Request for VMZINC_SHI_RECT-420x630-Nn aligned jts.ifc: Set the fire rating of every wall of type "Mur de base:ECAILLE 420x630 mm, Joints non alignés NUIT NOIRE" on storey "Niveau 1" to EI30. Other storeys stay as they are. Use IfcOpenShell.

First a look at what the model holds.

```python
import ifcopenshell
import ifcopenshell.util.element

model = ifcopenshell.open("VMZINC_SHI_RECT-420x630-Nn aligned jts.ifc")
print(model.schema)
storey = next(s for s in model.by_type("IfcBuildingStorey") if s.Name == "Niveau 1")
walls = [e for e in ifcopenshell.util.element.get_decomposition(storey) if e.is_a("IfcWall")]
seen = {}
for e in walls:
    element_type = ifcopenshell.util.element.get_type(e)
    key = (element_type.Name if element_type != e and element_type else None, ifcopenshell.util.element.get_pset(e, "Pset_WallCommon", "FireRating"))
    seen[key] = seen.get(key, 0) + 1
for (name, value), count in sorted(seen.items(), key=str):
    print(count, "x", name, "|", value)
```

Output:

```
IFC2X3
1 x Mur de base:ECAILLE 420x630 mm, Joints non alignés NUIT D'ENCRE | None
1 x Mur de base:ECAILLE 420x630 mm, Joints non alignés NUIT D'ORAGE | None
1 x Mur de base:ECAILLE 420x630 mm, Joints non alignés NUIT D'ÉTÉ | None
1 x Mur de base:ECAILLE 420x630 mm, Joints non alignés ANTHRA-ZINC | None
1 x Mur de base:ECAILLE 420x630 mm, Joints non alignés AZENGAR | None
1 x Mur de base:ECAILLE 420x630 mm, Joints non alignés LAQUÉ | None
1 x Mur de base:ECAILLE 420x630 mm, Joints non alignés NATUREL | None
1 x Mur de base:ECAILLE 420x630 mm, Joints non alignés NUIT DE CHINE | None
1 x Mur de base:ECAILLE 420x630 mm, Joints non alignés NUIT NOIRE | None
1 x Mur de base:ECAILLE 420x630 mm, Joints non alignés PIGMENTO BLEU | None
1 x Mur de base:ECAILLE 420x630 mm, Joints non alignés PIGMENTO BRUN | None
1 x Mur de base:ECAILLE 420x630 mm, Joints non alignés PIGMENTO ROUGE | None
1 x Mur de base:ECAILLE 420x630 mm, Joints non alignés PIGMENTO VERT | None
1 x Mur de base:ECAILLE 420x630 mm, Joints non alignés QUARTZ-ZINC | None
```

```python
import ifcopenshell
import ifcopenshell.api.pset
import ifcopenshell.util.element

model = ifcopenshell.open("VMZINC_SHI_RECT-420x630-Nn aligned jts.ifc")

storey = next(s for s in model.by_type("IfcBuildingStorey") if s.Name == "Niveau 1")
walls = [e for e in ifcopenshell.util.element.get_decomposition(storey) if e.is_a("IfcWall")]

count = 0
for e in walls:
    element_type = ifcopenshell.util.element.get_type(e)
    if element_type in (None, e) or element_type.Name != "Mur de base:ECAILLE 420x630 mm, Joints non alignés NUIT NOIRE":
        continue
    # add_pset returns the element's existing set when there is one.
    pset = ifcopenshell.api.pset.add_pset(model, product=e, name="Pset_WallCommon")
    ifcopenshell.api.pset.edit_pset(model, pset=pset, properties={"FireRating": "EI30"})
    count += 1

print(count, "walls updated")

model.write("VMZINC_SHI_RECT-420x630-Nn aligned jts_v2.ifc")
```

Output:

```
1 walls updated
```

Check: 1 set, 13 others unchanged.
